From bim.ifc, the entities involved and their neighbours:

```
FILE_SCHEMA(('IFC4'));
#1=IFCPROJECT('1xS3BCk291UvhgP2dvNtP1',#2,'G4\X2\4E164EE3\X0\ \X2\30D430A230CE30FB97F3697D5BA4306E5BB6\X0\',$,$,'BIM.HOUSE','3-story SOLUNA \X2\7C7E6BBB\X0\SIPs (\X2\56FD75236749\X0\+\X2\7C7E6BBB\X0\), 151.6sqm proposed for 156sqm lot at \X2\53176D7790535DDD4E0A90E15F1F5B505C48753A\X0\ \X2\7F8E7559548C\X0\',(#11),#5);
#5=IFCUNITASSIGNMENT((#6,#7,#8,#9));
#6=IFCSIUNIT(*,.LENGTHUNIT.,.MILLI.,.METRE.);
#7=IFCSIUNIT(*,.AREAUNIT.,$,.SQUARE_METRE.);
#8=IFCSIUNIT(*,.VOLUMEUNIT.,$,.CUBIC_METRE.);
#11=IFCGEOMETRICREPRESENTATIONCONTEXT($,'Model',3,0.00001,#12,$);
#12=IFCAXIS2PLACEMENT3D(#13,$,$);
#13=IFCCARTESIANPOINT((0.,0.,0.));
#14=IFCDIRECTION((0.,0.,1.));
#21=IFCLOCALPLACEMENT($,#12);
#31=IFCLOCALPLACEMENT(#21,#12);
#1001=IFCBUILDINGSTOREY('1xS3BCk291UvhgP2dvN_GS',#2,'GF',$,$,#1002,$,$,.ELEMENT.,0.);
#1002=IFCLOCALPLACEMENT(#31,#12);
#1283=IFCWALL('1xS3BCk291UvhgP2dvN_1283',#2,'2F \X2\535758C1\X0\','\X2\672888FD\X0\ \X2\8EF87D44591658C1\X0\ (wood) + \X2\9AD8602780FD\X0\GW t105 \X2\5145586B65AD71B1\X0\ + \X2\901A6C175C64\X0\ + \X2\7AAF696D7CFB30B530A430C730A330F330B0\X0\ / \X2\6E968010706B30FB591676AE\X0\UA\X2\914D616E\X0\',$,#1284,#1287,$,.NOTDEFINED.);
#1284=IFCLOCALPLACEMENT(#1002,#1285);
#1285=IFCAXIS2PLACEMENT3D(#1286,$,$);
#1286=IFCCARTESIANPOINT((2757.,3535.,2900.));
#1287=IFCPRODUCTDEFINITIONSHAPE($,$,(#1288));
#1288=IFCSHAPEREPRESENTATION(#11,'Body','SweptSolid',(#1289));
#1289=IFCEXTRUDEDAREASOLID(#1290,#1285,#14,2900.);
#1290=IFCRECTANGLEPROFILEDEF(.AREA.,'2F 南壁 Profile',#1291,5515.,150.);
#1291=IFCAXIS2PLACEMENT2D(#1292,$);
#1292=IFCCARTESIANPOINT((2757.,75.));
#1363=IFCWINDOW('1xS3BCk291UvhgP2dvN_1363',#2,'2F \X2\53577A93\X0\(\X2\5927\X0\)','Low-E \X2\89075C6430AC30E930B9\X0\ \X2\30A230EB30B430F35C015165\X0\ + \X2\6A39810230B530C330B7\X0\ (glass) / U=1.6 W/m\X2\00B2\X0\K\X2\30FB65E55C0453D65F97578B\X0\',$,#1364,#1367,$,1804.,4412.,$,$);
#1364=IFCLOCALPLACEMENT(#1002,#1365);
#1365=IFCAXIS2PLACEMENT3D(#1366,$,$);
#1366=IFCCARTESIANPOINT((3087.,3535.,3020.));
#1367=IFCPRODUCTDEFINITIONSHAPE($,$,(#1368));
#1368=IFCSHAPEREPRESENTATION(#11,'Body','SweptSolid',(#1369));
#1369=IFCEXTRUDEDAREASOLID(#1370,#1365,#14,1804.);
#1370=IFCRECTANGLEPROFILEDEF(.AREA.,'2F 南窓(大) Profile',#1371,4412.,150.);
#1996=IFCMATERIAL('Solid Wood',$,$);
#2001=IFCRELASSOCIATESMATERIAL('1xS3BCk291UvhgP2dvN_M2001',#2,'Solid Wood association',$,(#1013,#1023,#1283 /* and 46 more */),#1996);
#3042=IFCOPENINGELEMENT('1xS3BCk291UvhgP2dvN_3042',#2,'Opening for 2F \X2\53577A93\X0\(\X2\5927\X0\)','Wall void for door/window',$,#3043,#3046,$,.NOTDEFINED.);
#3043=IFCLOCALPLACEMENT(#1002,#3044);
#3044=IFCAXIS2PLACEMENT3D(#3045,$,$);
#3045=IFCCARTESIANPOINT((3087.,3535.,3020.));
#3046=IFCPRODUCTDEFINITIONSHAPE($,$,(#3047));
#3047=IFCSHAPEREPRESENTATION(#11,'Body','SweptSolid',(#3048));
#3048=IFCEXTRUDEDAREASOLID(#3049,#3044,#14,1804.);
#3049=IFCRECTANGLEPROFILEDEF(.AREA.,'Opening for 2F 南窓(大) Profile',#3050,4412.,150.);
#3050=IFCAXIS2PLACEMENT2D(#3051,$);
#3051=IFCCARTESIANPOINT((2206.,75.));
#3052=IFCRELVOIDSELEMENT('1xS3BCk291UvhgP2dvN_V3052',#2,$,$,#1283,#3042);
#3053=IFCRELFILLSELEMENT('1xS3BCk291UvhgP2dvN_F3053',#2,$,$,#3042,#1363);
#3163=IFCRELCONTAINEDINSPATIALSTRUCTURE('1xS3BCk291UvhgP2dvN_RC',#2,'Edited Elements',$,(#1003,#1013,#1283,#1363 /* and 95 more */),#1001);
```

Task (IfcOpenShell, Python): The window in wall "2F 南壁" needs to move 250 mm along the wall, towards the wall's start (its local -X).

```python
import ifcopenshell
import ifcopenshell.api.geometry
import ifcopenshell.util.placement

model = ifcopenshell.open("bim.ifc")

window = model.by_guid("1xS3BCk291UvhgP2dvN_1363")
opening = window.FillsVoids[0].RelatingOpeningElement
wall = opening.VoidsElements[0].RelatingBuildingElement

wall_matrix = ifcopenshell.util.placement.get_local_placement(wall.ObjectPlacement)
shift = wall_matrix[:3, 0] * -250.0
before = ifcopenshell.util.placement.get_local_placement(window.ObjectPlacement)[:3, 3].copy()

# The window is not placed relative to its opening, so move both.
for product in (opening, window):
    matrix = ifcopenshell.util.placement.get_local_placement(product.ObjectPlacement)
    matrix[:3, 3] += shift
    ifcopenshell.api.geometry.edit_object_placement(model, product=product, matrix=matrix, is_si=False)

after = ifcopenshell.util.placement.get_local_placement(window.ObjectPlacement)[:3, 3]
print("window moved by", (after - before).round(3) + 0.0)

model.write("bim-out.ifc")
```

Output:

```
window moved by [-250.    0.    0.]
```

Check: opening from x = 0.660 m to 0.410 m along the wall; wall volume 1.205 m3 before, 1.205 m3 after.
